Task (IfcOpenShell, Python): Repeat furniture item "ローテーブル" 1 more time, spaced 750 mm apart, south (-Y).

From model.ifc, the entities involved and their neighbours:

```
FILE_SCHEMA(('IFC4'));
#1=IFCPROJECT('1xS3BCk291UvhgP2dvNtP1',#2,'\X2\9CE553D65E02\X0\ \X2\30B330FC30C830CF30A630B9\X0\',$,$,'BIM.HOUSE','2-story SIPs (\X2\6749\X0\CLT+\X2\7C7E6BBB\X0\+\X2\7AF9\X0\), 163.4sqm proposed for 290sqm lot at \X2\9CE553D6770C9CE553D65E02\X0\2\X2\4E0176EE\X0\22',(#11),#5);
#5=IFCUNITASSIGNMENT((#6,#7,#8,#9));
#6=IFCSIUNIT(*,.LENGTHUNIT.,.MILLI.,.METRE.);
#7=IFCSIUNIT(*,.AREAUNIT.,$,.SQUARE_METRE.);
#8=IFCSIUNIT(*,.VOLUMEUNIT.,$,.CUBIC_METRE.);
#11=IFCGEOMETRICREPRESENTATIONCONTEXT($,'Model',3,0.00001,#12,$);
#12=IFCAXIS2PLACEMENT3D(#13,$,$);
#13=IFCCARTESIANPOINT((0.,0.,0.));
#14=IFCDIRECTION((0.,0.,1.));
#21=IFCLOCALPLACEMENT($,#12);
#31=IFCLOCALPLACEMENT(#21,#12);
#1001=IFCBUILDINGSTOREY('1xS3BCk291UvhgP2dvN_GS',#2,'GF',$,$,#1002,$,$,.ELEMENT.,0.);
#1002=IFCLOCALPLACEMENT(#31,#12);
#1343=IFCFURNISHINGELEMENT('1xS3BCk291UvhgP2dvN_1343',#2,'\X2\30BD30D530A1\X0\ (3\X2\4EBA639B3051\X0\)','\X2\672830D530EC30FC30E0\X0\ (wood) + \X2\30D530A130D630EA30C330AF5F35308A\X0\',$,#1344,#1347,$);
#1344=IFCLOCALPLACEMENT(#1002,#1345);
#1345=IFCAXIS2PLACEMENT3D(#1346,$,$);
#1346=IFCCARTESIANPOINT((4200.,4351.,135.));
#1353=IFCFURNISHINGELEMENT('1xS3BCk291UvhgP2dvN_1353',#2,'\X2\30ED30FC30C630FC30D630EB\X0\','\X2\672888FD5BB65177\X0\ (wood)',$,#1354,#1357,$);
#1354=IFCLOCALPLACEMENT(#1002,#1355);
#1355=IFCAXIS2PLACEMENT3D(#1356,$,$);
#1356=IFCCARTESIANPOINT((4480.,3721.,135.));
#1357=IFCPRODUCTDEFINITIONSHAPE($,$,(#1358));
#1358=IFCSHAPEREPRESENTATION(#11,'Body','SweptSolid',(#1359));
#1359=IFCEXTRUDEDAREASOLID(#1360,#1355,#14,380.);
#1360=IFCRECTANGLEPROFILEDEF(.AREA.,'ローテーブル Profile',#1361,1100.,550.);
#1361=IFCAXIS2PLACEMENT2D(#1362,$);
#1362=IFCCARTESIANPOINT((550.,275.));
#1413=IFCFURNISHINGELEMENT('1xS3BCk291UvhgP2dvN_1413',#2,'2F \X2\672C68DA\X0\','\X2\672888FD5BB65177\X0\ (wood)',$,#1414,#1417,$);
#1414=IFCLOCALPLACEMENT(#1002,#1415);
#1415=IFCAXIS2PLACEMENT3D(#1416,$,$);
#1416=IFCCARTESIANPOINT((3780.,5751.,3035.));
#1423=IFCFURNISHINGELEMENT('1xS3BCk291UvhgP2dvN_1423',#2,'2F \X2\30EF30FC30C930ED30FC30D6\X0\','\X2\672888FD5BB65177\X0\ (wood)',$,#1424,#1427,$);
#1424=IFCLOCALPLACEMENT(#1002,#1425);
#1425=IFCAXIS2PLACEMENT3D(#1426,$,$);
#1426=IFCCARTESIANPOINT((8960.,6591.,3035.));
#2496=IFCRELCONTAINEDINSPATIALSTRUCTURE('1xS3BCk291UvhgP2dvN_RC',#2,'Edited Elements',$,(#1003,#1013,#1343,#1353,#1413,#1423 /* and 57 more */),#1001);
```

```python
import numpy as np
import ifcopenshell
import ifcopenshell.api.geometry
import ifcopenshell.api.root
import ifcopenshell.util.element
import ifcopenshell.util.placement
import ifcopenshell.util.unit

model = ifcopenshell.open("model.ifc")
unit_scale = ifcopenshell.util.unit.calculate_unit_scale(model)


def reuse_history(source, copy):
    """copy_class also copies each property set's owner history, people and application; keep the originals."""
    for rel in copy.IsDefinedBy:
        if rel.is_a("IfcRelDefinesByProperties") and (history := rel.RelatingPropertyDefinition.OwnerHistory):
            rel.RelatingPropertyDefinition.OwnerHistory = source.OwnerHistory
            ifcopenshell.util.element.remove_deep2(model, history)


source = model.by_id(1353)
base = ifcopenshell.util.placement.get_local_placement(source.ObjectPlacement)
step = np.array([0.0, -1.0, 0.0]) * 0.75 / unit_scale

for i in range(1, 2):
    copy = ifcopenshell.api.root.copy_class(model, product=source)
    copy.Representation = ifcopenshell.util.element.copy_deep(
        model, source.Representation, exclude=["IfcGeometricRepresentationContext", "IfcRepresentationMap"]
    )
    reuse_history(source, copy)
    matrix = base.copy()
    matrix[:3, 3] += i * step
    print("added at", matrix[:3, 3].round(3) + 0.0)
    ifcopenshell.api.geometry.edit_object_placement(model, product=copy, matrix=matrix, is_si=False)

model.write("model-out.ifc")
```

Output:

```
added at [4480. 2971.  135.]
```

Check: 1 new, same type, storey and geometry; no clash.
